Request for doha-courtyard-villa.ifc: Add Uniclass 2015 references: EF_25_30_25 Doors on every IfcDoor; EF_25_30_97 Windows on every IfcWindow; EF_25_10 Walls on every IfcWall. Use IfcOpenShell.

First a look at what the model holds.

```python
import ifcopenshell

model = ifcopenshell.open("doha-courtyard-villa.ifc")
print(model.schema)
print("classifications:", [c.Name for c in model.by_type("IfcClassification")])
for ifc_class in ("IfcDoor", "IfcRoof", "IfcStair", "IfcWall", "IfcWindow"):
    print(ifc_class, len(model.by_type(ifc_class)))
```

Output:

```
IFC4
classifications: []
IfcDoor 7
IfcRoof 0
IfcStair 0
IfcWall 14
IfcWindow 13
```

```python
import ifcopenshell
import ifcopenshell.api.classification

model = ifcopenshell.open("doha-courtyard-villa.ifc")

system = ifcopenshell.api.classification.add_classification(model, classification="Uniclass 2015")

codes = {
    "IfcDoor": ("EF_25_30_25", "Doors"),
    "IfcWindow": ("EF_25_30_97", "Windows"),
    "IfcWall": ("EF_25_10", "Walls"),
}
for ifc_class, (code, name) in codes.items():
    products = model.by_type(ifc_class)
    ifcopenshell.api.classification.add_reference(
        model, products=products, classification=system, identification=code, name=name
    )
    print(code, len(products))

model.write("doha-courtyard-villa_v2.ifc")
```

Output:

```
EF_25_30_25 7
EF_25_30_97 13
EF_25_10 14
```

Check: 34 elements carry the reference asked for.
